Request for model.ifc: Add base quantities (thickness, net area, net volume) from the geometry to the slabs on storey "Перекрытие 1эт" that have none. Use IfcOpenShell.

First a look at what the model holds.

```python
import ifcopenshell
import ifcopenshell.util.element
import ifcopenshell.util.unit

model = ifcopenshell.open("model.ifc")
print(model.schema)
for unit_type in ("LENGTHUNIT", "AREAUNIT", "VOLUMEUNIT"):
    print(unit_type, ifcopenshell.util.unit.calculate_unit_scale(model, unit_type))
storey = next(s for s in model.by_type("IfcBuildingStorey") if s.Name == "Перекрытие 1эт")
slabs = [e for e in ifcopenshell.util.element.get_decomposition(storey) if e.is_a("IfcSlab")]
for e in sorted(slabs, key=lambda e: e.id()):
    print(e.id(), e.is_a(), e.Name, list(ifcopenshell.util.element.get_psets(e, qtos_only=True)), sep=" | ")
```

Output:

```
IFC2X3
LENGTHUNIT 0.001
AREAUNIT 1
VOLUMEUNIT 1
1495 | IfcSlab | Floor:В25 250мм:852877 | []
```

```python
import ifcopenshell
import ifcopenshell.api.pset
import ifcopenshell.geom
import ifcopenshell.util.element
import ifcopenshell.util.shape
import ifcopenshell.util.unit

model = ifcopenshell.open("model.ifc")
unit_scale = ifcopenshell.util.unit.calculate_unit_scale(model)
area_scale = ifcopenshell.util.unit.calculate_unit_scale(model, "AREAUNIT")
volume_scale = ifcopenshell.util.unit.calculate_unit_scale(model, "VOLUMEUNIT")
settings = ifcopenshell.geom.settings()

storey = next(s for s in model.by_type("IfcBuildingStorey") if s.Name == "Перекрытие 1эт")
slabs = [e for e in ifcopenshell.util.element.get_decomposition(storey) if e.is_a("IfcSlab")]

for e in sorted(slabs, key=lambda e: e.id()):
    if ifcopenshell.util.element.get_psets(e, qtos_only=True, should_inherit=False):
        continue
    # Geometry comes back in metres, in the element's own axes.
    shape = ifcopenshell.geom.create_shape(settings, e)
    values = {
        "Width": ifcopenshell.util.shape.get_z(shape.geometry) / unit_scale,
        "NetArea": ifcopenshell.util.shape.get_footprint_area(shape.geometry) / area_scale,
        "NetVolume": ifcopenshell.util.shape.get_volume(shape.geometry) / volume_scale,
    }
    qto = ifcopenshell.api.pset.add_qto(model, product=e, name="BaseQuantities")
    ifcopenshell.api.pset.edit_qto(model, qto=qto, properties=values)
    print(e.id(), {k: round(v, 3) for k, v in values.items()})

model.write("model_edited.ifc")
```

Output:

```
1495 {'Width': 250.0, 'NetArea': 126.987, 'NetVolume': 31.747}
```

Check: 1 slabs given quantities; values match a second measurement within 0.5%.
